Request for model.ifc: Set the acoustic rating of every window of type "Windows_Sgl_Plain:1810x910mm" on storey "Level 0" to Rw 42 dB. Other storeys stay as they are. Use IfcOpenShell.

First a look at what the model holds.

```python
import ifcopenshell
import ifcopenshell.util.element

model = ifcopenshell.open("model.ifc")
print(model.schema)
storey = next(s for s in model.by_type("IfcBuildingStorey") if s.Name == "Level 0")
windows = [e for e in ifcopenshell.util.element.get_decomposition(storey) if e.is_a("IfcWindow")]
seen = {}
for e in windows:
    element_type = ifcopenshell.util.element.get_type(e)
    key = (element_type.Name if element_type != e and element_type else None, ifcopenshell.util.element.get_pset(e, "Pset_WindowCommon", "AcousticRating"))
    seen[key] = seen.get(key, 0) + 1
for (name, value), count in sorted(seen.items(), key=str):
    print(count, "x", name, "|", value)
```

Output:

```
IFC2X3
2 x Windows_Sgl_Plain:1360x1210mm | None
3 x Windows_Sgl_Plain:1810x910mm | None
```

```python
import ifcopenshell
import ifcopenshell.api.pset
import ifcopenshell.util.element

model = ifcopenshell.open("model.ifc")

storey = next(s for s in model.by_type("IfcBuildingStorey") if s.Name == "Level 0")
windows = [e for e in ifcopenshell.util.element.get_decomposition(storey) if e.is_a("IfcWindow")]

count = 0
for e in windows:
    element_type = ifcopenshell.util.element.get_type(e)
    if element_type in (None, e) or element_type.Name != "Windows_Sgl_Plain:1810x910mm":
        continue
    # add_pset returns the element's existing set when there is one.
    pset = ifcopenshell.api.pset.add_pset(model, product=e, name="Pset_WindowCommon")
    ifcopenshell.api.pset.edit_pset(model, pset=pset, properties={"AcousticRating": "Rw 42 dB"})
    count += 1

print(count, "windows updated")

model.write("model_rev.ifc")
```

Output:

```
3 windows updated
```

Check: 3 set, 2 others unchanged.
